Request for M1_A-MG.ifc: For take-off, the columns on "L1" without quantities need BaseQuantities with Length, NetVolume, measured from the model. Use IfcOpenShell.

First a look at what the model holds.

```python
import ifcopenshell
import ifcopenshell.util.element
import ifcopenshell.util.unit

model = ifcopenshell.open("M1_A-MG.ifc")
print(model.schema)
for unit_type in ("LENGTHUNIT", "AREAUNIT", "VOLUMEUNIT"):
    print(unit_type, ifcopenshell.util.unit.calculate_unit_scale(model, unit_type))
storey = next(s for s in model.by_type("IfcBuildingStorey") if s.Name == "L1")
columns = [e for e in ifcopenshell.util.element.get_decomposition(storey) if e.is_a("IfcColumn")]
for e in sorted(columns, key=lambda e: e.id()):
    print(e.id(), e.is_a(), e.Name, list(ifcopenshell.util.element.get_psets(e, qtos_only=True)), sep=" | ")
```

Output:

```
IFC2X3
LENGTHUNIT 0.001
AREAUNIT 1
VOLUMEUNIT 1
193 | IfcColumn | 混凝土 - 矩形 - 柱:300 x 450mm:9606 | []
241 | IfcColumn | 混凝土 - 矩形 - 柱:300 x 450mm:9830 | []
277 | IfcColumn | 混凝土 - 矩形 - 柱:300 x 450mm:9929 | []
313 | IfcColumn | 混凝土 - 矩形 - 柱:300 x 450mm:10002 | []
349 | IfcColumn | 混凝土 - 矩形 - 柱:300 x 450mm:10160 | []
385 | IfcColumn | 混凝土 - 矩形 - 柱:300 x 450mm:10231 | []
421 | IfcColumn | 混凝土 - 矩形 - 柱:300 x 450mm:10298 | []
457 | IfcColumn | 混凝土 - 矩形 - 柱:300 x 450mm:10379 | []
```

```python
import ifcopenshell
import ifcopenshell.api.pset
import ifcopenshell.geom
import ifcopenshell.util.element
import ifcopenshell.util.shape
import ifcopenshell.util.unit

model = ifcopenshell.open("M1_A-MG.ifc")
unit_scale = ifcopenshell.util.unit.calculate_unit_scale(model)
volume_scale = ifcopenshell.util.unit.calculate_unit_scale(model, "VOLUMEUNIT")
settings = ifcopenshell.geom.settings()

storey = next(s for s in model.by_type("IfcBuildingStorey") if s.Name == "L1")
columns = [e for e in ifcopenshell.util.element.get_decomposition(storey) if e.is_a("IfcColumn")]

for e in sorted(columns, key=lambda e: e.id()):
    if ifcopenshell.util.element.get_psets(e, qtos_only=True, should_inherit=False):
        continue
    # Geometry comes back in metres, in the element's own axes.
    shape = ifcopenshell.geom.create_shape(settings, e)
    values = {
        "Length": ifcopenshell.util.shape.get_z(shape.geometry) / unit_scale,
        "NetVolume": ifcopenshell.util.shape.get_volume(shape.geometry) / volume_scale,
    }
    qto = ifcopenshell.api.pset.add_qto(model, product=e, name="BaseQuantities")
    ifcopenshell.api.pset.edit_qto(model, qto=qto, properties=values)
    print(e.id(), {k: round(v, 3) for k, v in values.items()})

model.write("M1_A-MG_updated.ifc")
```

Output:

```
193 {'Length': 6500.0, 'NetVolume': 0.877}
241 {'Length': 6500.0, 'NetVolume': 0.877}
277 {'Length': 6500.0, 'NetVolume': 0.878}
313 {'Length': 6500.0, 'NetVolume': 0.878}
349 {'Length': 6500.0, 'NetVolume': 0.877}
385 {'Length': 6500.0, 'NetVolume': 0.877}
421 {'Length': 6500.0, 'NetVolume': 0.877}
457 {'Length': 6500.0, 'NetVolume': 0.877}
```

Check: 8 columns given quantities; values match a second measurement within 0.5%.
